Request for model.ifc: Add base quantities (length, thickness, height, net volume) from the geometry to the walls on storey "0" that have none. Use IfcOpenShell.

First a look at what the model holds.

```python
import ifcopenshell
import ifcopenshell.util.element
import ifcopenshell.util.unit

model = ifcopenshell.open("model.ifc")
print(model.schema)
for unit_type in ("LENGTHUNIT", "AREAUNIT", "VOLUMEUNIT"):
    print(unit_type, ifcopenshell.util.unit.calculate_unit_scale(model, unit_type))
storey = next(s for s in model.by_type("IfcBuildingStorey") if s.Name == "0")
walls = [e for e in ifcopenshell.util.element.get_decomposition(storey) if e.is_a("IfcWall")]
for e in sorted(walls, key=lambda e: e.id()):
    print(e.id(), e.is_a(), e.Name, list(ifcopenshell.util.element.get_psets(e, qtos_only=True)), sep=" | ")
```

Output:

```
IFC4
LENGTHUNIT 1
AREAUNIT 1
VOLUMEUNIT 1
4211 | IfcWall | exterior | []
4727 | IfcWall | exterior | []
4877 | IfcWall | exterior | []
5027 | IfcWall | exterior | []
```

```python
import ifcopenshell
import ifcopenshell.api.pset
import ifcopenshell.geom
import ifcopenshell.util.element
import ifcopenshell.util.shape
import ifcopenshell.util.unit

model = ifcopenshell.open("model.ifc")
unit_scale = ifcopenshell.util.unit.calculate_unit_scale(model)
volume_scale = ifcopenshell.util.unit.calculate_unit_scale(model, "VOLUMEUNIT")
settings = ifcopenshell.geom.settings()

storey = next(s for s in model.by_type("IfcBuildingStorey") if s.Name == "0")
walls = [e for e in ifcopenshell.util.element.get_decomposition(storey) if e.is_a("IfcWall")]

for e in sorted(walls, key=lambda e: e.id()):
    if ifcopenshell.util.element.get_psets(e, qtos_only=True, should_inherit=False):
        continue
    # Geometry comes back in metres, in the element's own axes.
    shape = ifcopenshell.geom.create_shape(settings, e)
    values = {
        "Length": ifcopenshell.util.shape.get_x(shape.geometry) / unit_scale,
        "Width": ifcopenshell.util.shape.get_y(shape.geometry) / unit_scale,
        "Height": ifcopenshell.util.shape.get_z(shape.geometry) / unit_scale,
        "NetVolume": ifcopenshell.util.shape.get_volume(shape.geometry) / volume_scale,
    }
    qto = ifcopenshell.api.pset.add_qto(model, product=e, name="Qto_WallBaseQuantities")
    ifcopenshell.api.pset.edit_qto(model, qto=qto, properties=values)
    print(e.id(), {k: round(v, 3) for k, v in values.items()})

model.write("model_updated.ifc")
```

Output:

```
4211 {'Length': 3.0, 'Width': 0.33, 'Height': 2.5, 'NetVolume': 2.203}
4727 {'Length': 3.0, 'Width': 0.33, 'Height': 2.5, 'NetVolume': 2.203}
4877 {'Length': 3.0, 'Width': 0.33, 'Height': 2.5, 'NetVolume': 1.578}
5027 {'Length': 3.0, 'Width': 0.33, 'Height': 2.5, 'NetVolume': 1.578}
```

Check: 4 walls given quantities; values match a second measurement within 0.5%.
